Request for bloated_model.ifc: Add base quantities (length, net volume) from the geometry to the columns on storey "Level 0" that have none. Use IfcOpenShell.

First a look at what the model holds.

```python
import ifcopenshell
import ifcopenshell.util.element
import ifcopenshell.util.unit

model = ifcopenshell.open("bloated_model.ifc")
print(model.schema)
for unit_type in ("LENGTHUNIT", "AREAUNIT", "VOLUMEUNIT"):
    print(unit_type, ifcopenshell.util.unit.calculate_unit_scale(model, unit_type))
storey = next(s for s in model.by_type("IfcBuildingStorey") if s.Name == "Level 0")
columns = [e for e in ifcopenshell.util.element.get_decomposition(storey) if e.is_a("IfcColumn")]
for e in sorted(columns, key=lambda e: e.id()):
    print(e.id(), e.is_a(), e.Name, list(ifcopenshell.util.element.get_psets(e, qtos_only=True)), sep=" | ")
```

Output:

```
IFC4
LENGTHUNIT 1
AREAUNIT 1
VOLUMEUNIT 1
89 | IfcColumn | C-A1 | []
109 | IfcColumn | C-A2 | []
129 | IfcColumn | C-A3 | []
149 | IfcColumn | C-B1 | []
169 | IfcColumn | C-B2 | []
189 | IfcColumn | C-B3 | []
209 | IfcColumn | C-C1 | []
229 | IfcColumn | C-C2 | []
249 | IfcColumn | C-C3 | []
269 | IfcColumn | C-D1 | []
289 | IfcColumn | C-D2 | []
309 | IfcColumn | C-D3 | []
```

```python
import ifcopenshell
import ifcopenshell.api.pset
import ifcopenshell.geom
import ifcopenshell.util.element
import ifcopenshell.util.shape
import ifcopenshell.util.unit

model = ifcopenshell.open("bloated_model.ifc")
unit_scale = ifcopenshell.util.unit.calculate_unit_scale(model)
volume_scale = ifcopenshell.util.unit.calculate_unit_scale(model, "VOLUMEUNIT")
settings = ifcopenshell.geom.settings()

storey = next(s for s in model.by_type("IfcBuildingStorey") if s.Name == "Level 0")
columns = [e for e in ifcopenshell.util.element.get_decomposition(storey) if e.is_a("IfcColumn")]

for e in sorted(columns, key=lambda e: e.id()):
    if ifcopenshell.util.element.get_psets(e, qtos_only=True, should_inherit=False):
        continue
    # Geometry comes back in metres, in the element's own axes.
    shape = ifcopenshell.geom.create_shape(settings, e)
    values = {
        "Length": ifcopenshell.util.shape.get_z(shape.geometry) / unit_scale,
        "NetVolume": ifcopenshell.util.shape.get_volume(shape.geometry) / volume_scale,
    }
    qto = ifcopenshell.api.pset.add_qto(model, product=e, name="Qto_ColumnBaseQuantities")
    ifcopenshell.api.pset.edit_qto(model, qto=qto, properties=values)
    print(e.id(), {k: round(v, 3) for k, v in values.items()})

model.write("bloated_model_v2.ifc")
```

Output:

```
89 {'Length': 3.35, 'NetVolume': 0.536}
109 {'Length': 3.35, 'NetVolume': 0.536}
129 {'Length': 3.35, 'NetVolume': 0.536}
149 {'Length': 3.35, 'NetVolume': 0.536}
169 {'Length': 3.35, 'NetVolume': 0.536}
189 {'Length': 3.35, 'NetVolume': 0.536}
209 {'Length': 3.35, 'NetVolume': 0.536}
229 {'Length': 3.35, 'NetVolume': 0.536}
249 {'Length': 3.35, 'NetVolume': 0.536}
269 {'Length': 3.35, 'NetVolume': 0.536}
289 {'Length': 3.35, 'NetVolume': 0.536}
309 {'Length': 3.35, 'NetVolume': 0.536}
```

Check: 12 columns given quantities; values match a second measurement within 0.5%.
